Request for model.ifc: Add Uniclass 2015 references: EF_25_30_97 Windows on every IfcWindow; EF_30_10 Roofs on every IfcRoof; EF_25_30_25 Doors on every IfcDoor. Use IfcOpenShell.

First a look at what the model holds.

```python
import ifcopenshell

model = ifcopenshell.open("model.ifc")
print(model.schema)
print("classifications:", [c.Name for c in model.by_type("IfcClassification")])
for ifc_class in ("IfcDoor", "IfcRoof", "IfcStair", "IfcWall", "IfcWindow"):
    print(ifc_class, len(model.by_type(ifc_class)))
```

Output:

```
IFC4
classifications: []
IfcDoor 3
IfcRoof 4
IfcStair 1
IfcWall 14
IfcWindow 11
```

```python
import ifcopenshell
import ifcopenshell.api.classification

model = ifcopenshell.open("model.ifc")

system = ifcopenshell.api.classification.add_classification(model, classification="Uniclass 2015")

codes = {
    "IfcWindow": ("EF_25_30_97", "Windows"),
    "IfcRoof": ("EF_30_10", "Roofs"),
    "IfcDoor": ("EF_25_30_25", "Doors"),
}
for ifc_class, (code, name) in codes.items():
    products = model.by_type(ifc_class)
    ifcopenshell.api.classification.add_reference(
        model, products=products, classification=system, identification=code, name=name
    )
    print(code, len(products))

model.write("model_rev.ifc")
```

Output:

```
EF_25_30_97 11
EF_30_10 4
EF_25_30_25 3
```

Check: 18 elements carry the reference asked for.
